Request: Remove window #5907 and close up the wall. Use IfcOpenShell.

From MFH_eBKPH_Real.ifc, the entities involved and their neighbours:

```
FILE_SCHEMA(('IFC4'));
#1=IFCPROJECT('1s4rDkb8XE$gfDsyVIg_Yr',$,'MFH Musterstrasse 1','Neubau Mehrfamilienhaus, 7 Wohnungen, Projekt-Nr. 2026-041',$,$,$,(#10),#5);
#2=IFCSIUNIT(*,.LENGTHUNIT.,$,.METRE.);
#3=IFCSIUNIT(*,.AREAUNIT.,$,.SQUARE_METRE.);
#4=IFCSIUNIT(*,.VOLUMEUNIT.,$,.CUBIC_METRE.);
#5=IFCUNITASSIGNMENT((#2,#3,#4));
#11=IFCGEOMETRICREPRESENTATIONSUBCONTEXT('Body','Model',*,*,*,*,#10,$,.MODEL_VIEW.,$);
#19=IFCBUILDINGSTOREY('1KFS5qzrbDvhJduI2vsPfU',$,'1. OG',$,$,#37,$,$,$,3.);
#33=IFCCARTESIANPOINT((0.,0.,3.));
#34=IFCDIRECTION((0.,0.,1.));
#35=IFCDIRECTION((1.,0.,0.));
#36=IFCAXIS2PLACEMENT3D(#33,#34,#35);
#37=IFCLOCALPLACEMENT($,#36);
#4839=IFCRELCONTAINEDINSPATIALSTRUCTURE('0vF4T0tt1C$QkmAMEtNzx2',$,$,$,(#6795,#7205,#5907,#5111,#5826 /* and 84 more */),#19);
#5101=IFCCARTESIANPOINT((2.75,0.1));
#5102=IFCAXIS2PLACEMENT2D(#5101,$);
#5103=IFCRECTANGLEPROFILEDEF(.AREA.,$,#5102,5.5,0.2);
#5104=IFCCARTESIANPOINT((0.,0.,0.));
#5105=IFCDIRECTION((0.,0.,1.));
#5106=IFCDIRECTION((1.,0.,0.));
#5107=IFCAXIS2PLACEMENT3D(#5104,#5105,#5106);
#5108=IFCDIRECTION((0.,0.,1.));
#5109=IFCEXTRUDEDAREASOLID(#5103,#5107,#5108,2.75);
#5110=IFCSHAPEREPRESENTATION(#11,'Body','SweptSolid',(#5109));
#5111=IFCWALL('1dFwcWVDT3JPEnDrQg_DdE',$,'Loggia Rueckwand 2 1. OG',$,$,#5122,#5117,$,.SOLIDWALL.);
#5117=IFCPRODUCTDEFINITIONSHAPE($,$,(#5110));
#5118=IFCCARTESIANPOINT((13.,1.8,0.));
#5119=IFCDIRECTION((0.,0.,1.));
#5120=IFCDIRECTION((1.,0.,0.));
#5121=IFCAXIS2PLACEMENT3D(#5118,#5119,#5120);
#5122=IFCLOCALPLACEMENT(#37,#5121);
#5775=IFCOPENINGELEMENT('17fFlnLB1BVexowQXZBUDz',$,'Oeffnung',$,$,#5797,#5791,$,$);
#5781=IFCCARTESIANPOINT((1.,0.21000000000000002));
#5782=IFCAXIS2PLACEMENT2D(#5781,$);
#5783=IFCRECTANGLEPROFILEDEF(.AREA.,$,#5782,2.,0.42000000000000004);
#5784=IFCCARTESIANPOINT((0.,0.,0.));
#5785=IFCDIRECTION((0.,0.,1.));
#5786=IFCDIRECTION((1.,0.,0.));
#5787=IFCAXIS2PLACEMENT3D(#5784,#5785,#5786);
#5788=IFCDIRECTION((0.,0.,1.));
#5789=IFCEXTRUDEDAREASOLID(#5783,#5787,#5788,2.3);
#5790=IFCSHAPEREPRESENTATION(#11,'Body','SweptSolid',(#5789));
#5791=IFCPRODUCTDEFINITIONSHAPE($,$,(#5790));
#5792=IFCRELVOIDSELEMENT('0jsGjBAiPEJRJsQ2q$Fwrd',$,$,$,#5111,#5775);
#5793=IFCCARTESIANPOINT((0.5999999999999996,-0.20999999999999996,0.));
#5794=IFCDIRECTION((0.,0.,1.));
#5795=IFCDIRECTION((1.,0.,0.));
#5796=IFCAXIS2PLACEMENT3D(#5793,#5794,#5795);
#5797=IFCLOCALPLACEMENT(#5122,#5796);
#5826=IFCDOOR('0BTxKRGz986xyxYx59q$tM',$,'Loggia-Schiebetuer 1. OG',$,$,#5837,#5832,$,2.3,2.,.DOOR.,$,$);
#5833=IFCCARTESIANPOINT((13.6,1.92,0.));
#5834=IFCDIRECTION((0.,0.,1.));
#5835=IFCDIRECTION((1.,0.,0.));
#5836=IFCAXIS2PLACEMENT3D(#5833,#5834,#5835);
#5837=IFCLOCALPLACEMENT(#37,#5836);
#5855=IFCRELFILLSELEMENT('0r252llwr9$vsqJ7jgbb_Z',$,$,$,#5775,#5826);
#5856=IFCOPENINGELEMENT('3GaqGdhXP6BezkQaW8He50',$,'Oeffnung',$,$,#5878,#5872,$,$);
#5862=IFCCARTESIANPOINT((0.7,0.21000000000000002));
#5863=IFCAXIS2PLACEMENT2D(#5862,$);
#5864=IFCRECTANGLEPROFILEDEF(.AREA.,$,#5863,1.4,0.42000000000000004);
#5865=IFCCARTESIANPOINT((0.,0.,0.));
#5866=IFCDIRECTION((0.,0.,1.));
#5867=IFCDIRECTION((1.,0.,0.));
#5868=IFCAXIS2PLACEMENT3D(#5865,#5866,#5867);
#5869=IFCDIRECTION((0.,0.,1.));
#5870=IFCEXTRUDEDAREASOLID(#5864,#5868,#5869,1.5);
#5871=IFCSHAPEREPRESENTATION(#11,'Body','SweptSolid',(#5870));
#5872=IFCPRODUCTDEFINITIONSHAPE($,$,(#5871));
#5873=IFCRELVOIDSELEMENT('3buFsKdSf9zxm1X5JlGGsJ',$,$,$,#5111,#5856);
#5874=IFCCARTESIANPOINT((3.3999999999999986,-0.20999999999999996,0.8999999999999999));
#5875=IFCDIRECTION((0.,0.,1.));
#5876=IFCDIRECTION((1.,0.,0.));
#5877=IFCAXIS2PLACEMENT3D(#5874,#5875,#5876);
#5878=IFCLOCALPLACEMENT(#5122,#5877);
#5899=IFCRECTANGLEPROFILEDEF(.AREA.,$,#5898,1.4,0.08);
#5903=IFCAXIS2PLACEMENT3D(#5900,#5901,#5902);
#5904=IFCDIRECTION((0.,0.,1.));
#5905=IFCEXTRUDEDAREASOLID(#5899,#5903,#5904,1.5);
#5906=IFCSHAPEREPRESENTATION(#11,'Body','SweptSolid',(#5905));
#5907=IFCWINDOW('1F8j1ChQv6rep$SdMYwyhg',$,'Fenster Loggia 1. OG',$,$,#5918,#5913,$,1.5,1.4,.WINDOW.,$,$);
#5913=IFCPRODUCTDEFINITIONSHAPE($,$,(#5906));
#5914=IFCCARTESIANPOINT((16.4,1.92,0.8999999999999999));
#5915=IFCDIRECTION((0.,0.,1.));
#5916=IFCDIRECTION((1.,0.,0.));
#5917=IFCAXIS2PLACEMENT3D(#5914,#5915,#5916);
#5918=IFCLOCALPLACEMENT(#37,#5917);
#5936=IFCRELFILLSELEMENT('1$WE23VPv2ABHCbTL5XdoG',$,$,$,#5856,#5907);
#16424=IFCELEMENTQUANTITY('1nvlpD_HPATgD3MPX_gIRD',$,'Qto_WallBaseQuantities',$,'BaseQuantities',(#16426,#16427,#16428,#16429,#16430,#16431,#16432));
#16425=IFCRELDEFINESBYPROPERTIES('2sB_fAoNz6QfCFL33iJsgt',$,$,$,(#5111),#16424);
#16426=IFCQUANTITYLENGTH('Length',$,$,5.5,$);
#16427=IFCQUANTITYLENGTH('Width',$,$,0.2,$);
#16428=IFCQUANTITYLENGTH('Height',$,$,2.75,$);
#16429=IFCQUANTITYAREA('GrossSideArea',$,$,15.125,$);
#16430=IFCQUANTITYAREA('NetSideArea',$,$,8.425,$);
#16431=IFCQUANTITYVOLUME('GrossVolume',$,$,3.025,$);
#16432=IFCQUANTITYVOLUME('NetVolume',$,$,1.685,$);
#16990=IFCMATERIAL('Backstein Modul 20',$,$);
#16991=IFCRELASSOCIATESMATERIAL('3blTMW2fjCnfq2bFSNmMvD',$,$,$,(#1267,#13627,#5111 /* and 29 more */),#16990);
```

```python
import ifcopenshell
import ifcopenshell.api.feature
import ifcopenshell.api.pset
import ifcopenshell.api.root
import ifcopenshell.geom
import ifcopenshell.util.element
import ifcopenshell.util.shape
import ifcopenshell.util.unit

model = ifcopenshell.open("MFH_eBKPH_Real.ifc")
area_scale = ifcopenshell.util.unit.calculate_unit_scale(model, "AREAUNIT")
volume_scale = ifcopenshell.util.unit.calculate_unit_scale(model, "VOLUMEUNIT")
settings = ifcopenshell.geom.settings()


def volume(element):
    """Net volume in cubic metres, openings subtracted."""
    shape = ifcopenshell.geom.create_shape(settings, element)
    return ifcopenshell.util.shape.get_volume(shape.geometry)


window = model.by_guid("1F8j1ChQv6rep$SdMYwyhg")
opening = window.FillsVoids[0].RelatingOpeningElement
wall = opening.VoidsElements[0].RelatingBuildingElement
before = volume(wall)

ifcopenshell.api.root.remove_product(model, product=window)
ifcopenshell.api.feature.remove_feature(model, feature=opening)

after = volume(wall)
thickness = 0.2  # wall thickness in metres

# Update the wall's stored quantities.
qto = model.by_id(ifcopenshell.util.element.get_pset(wall, "Qto_WallBaseQuantities", should_inherit=False)["id"])
ifcopenshell.api.pset.edit_qto(model, qto=qto, properties={
    "NetSideArea": after / thickness / area_scale,
    "NetVolume": after / volume_scale,
})

print(f"wall volume {before:.3f} -> {after:.3f} m3")

model.write("MFH_eBKPH_Real-out.ifc")
```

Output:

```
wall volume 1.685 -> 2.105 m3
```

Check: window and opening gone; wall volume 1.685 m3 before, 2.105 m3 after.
